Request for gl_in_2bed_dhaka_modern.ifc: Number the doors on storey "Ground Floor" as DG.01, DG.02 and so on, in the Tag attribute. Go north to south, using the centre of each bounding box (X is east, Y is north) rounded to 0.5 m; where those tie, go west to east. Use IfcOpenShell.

First a look at what the model holds.

```python
import ifcopenshell
import ifcopenshell.util.element
import ifcopenshell.util.placement

model = ifcopenshell.open("gl_in_2bed_dhaka_modern.ifc")
print(model.schema)
storey = next(s for s in model.by_type("IfcBuildingStorey") if s.Name == "Ground Floor")
doors = [e for e in ifcopenshell.util.element.get_decomposition(storey) if e.is_a("IfcDoor")]
for e in sorted(doors, key=lambda e: e.id()):
    origin = ifcopenshell.util.placement.get_local_placement(e.ObjectPlacement)[:3, 3]
    print(e.id(), e.Tag, e.Name, origin.round(2) + 0.0, sep=" | ")
```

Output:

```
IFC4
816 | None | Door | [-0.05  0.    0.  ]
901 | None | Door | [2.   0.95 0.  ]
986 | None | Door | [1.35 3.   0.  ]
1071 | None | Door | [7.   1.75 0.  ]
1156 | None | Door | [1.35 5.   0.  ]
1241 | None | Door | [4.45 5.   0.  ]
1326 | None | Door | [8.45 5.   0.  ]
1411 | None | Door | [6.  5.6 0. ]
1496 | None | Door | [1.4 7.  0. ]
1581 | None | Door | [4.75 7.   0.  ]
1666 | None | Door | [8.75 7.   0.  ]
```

```python
import ifcopenshell
import ifcopenshell.geom
import ifcopenshell.util.element
import ifcopenshell.util.shape

model = ifcopenshell.open("gl_in_2bed_dhaka_modern.ifc")
settings = ifcopenshell.geom.settings()
settings.set("use-world-coords", True)


def centre(element):
    shape = ifcopenshell.geom.create_shape(settings, element)
    return ifcopenshell.util.shape.get_bbox_centroid(shape.geometry)


storey = next(s for s in model.by_type("IfcBuildingStorey") if s.Name == "Ground Floor")
doors = [e for e in ifcopenshell.util.element.get_decomposition(storey) if e.is_a("IfcDoor")]

# Insertion points can sit at a corner or the storey origin, so sort by the geometry (in metres).
centres = {e: centre(e) for e in doors}
doors.sort(key=lambda e: (-round(centres[e][1] / 0.5), centres[e][0]))

for i, e in enumerate(doors, start=1):
    number = f"DG.{i:02d}"
    e.Tag = number
    print(e.id(), number)

model.write("gl_in_2bed_dhaka_modern_v2.ifc")
```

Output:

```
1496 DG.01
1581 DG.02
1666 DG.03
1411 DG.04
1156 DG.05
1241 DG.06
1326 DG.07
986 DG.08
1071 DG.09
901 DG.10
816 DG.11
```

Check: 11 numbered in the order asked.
